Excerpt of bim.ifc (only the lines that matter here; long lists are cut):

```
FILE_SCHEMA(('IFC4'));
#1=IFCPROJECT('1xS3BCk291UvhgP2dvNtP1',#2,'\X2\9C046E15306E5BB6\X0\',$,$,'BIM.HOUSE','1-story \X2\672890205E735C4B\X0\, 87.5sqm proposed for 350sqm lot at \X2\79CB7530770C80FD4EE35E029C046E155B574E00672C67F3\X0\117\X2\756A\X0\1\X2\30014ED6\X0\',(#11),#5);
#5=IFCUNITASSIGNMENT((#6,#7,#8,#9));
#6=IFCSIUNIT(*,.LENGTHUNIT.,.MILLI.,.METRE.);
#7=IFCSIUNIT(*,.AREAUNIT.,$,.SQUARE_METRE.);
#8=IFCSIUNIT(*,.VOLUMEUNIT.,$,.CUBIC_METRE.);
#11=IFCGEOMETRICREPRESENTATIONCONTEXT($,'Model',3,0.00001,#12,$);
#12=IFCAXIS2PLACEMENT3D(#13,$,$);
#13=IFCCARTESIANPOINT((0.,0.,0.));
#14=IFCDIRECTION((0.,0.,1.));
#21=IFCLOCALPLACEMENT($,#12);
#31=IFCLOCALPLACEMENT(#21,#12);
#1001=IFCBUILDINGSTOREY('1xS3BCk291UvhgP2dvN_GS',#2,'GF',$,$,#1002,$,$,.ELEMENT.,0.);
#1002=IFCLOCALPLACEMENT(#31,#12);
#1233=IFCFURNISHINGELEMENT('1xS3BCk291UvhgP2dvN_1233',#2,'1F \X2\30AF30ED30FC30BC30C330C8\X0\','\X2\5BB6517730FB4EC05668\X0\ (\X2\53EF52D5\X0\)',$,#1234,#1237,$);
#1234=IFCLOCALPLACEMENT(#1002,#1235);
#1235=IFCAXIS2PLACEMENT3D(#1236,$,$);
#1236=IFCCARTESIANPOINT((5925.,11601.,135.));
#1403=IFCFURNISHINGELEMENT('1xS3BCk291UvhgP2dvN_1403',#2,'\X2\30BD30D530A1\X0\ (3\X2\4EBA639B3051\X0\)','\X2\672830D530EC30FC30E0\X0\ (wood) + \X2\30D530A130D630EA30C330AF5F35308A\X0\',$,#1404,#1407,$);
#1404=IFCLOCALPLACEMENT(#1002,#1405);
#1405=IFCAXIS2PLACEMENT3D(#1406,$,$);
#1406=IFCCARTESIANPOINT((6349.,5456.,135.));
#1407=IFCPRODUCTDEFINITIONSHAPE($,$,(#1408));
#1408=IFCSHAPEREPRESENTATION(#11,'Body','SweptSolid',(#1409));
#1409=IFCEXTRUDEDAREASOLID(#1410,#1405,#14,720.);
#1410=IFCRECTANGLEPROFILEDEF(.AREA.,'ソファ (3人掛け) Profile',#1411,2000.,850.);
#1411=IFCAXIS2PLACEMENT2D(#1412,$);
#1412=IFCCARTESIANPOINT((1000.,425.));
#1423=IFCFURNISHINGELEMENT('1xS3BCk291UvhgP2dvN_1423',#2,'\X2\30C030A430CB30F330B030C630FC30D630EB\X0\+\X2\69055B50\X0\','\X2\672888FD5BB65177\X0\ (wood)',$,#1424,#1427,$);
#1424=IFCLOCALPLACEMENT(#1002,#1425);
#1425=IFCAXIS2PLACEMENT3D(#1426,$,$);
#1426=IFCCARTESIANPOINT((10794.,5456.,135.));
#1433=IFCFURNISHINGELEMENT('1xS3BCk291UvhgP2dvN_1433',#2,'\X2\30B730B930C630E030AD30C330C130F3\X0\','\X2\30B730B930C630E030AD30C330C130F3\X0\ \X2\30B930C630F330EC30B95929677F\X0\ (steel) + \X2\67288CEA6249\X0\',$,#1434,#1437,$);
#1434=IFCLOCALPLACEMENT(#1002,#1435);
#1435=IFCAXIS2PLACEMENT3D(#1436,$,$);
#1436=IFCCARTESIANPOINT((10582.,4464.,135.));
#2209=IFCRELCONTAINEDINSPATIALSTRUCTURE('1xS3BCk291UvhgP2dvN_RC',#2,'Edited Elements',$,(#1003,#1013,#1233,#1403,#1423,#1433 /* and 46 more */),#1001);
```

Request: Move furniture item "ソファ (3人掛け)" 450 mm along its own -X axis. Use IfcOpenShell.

```python
import ifcopenshell
import ifcopenshell.api.geometry
import ifcopenshell.util.placement
import ifcopenshell.util.unit

model = ifcopenshell.open("bim.ifc")
unit_scale = ifcopenshell.util.unit.calculate_unit_scale(model)

item = model.by_guid("1xS3BCk291UvhgP2dvN_1403")
matrix = ifcopenshell.util.placement.get_local_placement(item.ObjectPlacement)
matrix[:3, 3] -= matrix[:3, 0] * 0.45 / unit_scale
ifcopenshell.api.geometry.edit_object_placement(model, product=item, matrix=matrix, is_si=False)

print(ifcopenshell.util.placement.get_local_placement(item.ObjectPlacement).round(3) + 0.0)

model.write("bim_v2.ifc")
```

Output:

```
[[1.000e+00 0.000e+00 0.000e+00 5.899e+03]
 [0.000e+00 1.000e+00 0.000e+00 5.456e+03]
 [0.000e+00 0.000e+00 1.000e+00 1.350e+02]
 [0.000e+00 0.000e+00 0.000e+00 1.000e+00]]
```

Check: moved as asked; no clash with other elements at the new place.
